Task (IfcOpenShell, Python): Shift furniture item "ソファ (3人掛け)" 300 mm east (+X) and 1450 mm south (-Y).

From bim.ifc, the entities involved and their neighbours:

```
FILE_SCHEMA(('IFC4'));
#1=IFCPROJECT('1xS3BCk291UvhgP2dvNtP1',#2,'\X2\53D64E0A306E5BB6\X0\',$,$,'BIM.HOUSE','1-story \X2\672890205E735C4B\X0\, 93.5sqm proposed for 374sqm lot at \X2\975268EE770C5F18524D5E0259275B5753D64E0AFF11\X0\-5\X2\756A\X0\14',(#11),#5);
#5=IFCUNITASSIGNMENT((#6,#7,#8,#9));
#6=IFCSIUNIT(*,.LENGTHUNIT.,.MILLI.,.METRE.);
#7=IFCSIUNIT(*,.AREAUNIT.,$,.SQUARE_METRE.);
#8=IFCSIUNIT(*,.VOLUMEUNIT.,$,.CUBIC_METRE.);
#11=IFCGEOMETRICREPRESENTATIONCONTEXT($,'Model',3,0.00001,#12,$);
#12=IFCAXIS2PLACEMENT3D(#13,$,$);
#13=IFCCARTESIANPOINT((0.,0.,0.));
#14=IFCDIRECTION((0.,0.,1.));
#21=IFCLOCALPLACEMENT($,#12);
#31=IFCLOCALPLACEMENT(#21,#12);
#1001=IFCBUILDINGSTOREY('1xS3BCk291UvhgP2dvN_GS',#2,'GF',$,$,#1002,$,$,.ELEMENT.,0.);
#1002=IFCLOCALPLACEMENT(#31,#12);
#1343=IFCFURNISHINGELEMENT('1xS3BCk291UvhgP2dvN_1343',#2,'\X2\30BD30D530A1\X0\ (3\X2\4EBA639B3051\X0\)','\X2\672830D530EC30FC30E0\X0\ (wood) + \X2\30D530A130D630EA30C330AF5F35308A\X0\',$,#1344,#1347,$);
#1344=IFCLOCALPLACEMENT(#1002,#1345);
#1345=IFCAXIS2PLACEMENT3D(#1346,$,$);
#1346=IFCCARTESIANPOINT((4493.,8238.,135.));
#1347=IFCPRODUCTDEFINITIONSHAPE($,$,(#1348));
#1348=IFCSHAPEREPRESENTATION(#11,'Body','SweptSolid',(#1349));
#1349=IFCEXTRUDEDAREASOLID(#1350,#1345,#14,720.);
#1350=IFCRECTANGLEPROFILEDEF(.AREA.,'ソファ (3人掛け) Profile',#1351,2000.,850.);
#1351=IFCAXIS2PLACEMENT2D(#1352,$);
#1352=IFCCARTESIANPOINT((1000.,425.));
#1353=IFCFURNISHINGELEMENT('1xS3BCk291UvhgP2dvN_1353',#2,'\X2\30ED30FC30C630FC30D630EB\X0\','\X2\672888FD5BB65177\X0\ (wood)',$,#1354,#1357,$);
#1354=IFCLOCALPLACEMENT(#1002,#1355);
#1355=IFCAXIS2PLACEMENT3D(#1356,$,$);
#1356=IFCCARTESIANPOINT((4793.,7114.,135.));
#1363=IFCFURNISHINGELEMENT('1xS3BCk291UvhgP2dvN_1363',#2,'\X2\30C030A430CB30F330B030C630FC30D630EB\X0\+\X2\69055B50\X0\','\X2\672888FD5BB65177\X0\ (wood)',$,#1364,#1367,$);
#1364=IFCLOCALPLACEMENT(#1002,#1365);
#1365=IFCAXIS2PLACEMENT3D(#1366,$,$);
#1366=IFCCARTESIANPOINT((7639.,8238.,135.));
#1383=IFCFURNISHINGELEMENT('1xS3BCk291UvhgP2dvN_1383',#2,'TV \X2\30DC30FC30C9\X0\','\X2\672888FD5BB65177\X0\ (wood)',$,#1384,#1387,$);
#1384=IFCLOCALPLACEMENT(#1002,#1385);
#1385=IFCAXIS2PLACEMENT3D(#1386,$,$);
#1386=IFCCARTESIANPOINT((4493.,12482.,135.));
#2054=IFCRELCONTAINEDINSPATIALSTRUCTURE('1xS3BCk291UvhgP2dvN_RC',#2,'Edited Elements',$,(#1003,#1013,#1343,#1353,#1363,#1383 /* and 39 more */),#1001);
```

```python
import ifcopenshell
import ifcopenshell.api.geometry
import ifcopenshell.util.placement
import ifcopenshell.util.unit

model = ifcopenshell.open("bim.ifc")
unit_scale = ifcopenshell.util.unit.calculate_unit_scale(model)

item = model.by_guid("1xS3BCk291UvhgP2dvN_1343")
matrix = ifcopenshell.util.placement.get_local_placement(item.ObjectPlacement)
matrix[0, 3] += 0.3 / unit_scale
matrix[1, 3] -= 1.45 / unit_scale
ifcopenshell.api.geometry.edit_object_placement(model, product=item, matrix=matrix, is_si=False)

print(ifcopenshell.util.placement.get_local_placement(item.ObjectPlacement).round(3) + 0.0)

model.write("bim_updated.ifc")
```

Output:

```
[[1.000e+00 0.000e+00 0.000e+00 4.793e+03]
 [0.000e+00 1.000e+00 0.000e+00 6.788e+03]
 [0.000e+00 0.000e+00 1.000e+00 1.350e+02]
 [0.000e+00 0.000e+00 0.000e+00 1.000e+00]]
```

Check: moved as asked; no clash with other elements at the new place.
